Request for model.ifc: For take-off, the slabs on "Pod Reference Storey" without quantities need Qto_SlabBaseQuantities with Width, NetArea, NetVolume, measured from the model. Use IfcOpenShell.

First a look at what the model holds.

```python
import ifcopenshell
import ifcopenshell.util.element
import ifcopenshell.util.unit

model = ifcopenshell.open("model.ifc")
print(model.schema)
for unit_type in ("LENGTHUNIT", "AREAUNIT", "VOLUMEUNIT"):
    print(unit_type, ifcopenshell.util.unit.calculate_unit_scale(model, unit_type))
storey = next(s for s in model.by_type("IfcBuildingStorey") if s.Name == "Pod Reference Storey")
slabs = [e for e in ifcopenshell.util.element.get_decomposition(storey) if e.is_a("IfcSlab")]
for e in sorted(slabs, key=lambda e: e.id()):
    print(e.id(), e.is_a(), e.Name, list(ifcopenshell.util.element.get_psets(e, qtos_only=True)), sep=" | ")
```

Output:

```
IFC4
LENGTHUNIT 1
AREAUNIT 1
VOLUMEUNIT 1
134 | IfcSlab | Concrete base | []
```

```python
import ifcopenshell
import ifcopenshell.api.pset
import ifcopenshell.geom
import ifcopenshell.util.element
import ifcopenshell.util.shape
import ifcopenshell.util.unit

model = ifcopenshell.open("model.ifc")
unit_scale = ifcopenshell.util.unit.calculate_unit_scale(model)
area_scale = ifcopenshell.util.unit.calculate_unit_scale(model, "AREAUNIT")
volume_scale = ifcopenshell.util.unit.calculate_unit_scale(model, "VOLUMEUNIT")
settings = ifcopenshell.geom.settings()

storey = next(s for s in model.by_type("IfcBuildingStorey") if s.Name == "Pod Reference Storey")
slabs = [e for e in ifcopenshell.util.element.get_decomposition(storey) if e.is_a("IfcSlab")]

for e in sorted(slabs, key=lambda e: e.id()):
    if ifcopenshell.util.element.get_psets(e, qtos_only=True, should_inherit=False):
        continue
    # Geometry comes back in metres, in the element's own axes.
    shape = ifcopenshell.geom.create_shape(settings, e)
    values = {
        "Width": ifcopenshell.util.shape.get_z(shape.geometry) / unit_scale,
        "NetArea": ifcopenshell.util.shape.get_footprint_area(shape.geometry) / area_scale,
        "NetVolume": ifcopenshell.util.shape.get_volume(shape.geometry) / volume_scale,
    }
    qto = ifcopenshell.api.pset.add_qto(model, product=e, name="Qto_SlabBaseQuantities")
    ifcopenshell.api.pset.edit_qto(model, qto=qto, properties=values)
    print(e.id(), {k: round(v, 3) for k, v in values.items()})

model.write("model_rev.ifc")
```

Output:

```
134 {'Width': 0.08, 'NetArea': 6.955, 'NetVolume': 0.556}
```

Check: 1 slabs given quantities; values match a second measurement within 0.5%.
